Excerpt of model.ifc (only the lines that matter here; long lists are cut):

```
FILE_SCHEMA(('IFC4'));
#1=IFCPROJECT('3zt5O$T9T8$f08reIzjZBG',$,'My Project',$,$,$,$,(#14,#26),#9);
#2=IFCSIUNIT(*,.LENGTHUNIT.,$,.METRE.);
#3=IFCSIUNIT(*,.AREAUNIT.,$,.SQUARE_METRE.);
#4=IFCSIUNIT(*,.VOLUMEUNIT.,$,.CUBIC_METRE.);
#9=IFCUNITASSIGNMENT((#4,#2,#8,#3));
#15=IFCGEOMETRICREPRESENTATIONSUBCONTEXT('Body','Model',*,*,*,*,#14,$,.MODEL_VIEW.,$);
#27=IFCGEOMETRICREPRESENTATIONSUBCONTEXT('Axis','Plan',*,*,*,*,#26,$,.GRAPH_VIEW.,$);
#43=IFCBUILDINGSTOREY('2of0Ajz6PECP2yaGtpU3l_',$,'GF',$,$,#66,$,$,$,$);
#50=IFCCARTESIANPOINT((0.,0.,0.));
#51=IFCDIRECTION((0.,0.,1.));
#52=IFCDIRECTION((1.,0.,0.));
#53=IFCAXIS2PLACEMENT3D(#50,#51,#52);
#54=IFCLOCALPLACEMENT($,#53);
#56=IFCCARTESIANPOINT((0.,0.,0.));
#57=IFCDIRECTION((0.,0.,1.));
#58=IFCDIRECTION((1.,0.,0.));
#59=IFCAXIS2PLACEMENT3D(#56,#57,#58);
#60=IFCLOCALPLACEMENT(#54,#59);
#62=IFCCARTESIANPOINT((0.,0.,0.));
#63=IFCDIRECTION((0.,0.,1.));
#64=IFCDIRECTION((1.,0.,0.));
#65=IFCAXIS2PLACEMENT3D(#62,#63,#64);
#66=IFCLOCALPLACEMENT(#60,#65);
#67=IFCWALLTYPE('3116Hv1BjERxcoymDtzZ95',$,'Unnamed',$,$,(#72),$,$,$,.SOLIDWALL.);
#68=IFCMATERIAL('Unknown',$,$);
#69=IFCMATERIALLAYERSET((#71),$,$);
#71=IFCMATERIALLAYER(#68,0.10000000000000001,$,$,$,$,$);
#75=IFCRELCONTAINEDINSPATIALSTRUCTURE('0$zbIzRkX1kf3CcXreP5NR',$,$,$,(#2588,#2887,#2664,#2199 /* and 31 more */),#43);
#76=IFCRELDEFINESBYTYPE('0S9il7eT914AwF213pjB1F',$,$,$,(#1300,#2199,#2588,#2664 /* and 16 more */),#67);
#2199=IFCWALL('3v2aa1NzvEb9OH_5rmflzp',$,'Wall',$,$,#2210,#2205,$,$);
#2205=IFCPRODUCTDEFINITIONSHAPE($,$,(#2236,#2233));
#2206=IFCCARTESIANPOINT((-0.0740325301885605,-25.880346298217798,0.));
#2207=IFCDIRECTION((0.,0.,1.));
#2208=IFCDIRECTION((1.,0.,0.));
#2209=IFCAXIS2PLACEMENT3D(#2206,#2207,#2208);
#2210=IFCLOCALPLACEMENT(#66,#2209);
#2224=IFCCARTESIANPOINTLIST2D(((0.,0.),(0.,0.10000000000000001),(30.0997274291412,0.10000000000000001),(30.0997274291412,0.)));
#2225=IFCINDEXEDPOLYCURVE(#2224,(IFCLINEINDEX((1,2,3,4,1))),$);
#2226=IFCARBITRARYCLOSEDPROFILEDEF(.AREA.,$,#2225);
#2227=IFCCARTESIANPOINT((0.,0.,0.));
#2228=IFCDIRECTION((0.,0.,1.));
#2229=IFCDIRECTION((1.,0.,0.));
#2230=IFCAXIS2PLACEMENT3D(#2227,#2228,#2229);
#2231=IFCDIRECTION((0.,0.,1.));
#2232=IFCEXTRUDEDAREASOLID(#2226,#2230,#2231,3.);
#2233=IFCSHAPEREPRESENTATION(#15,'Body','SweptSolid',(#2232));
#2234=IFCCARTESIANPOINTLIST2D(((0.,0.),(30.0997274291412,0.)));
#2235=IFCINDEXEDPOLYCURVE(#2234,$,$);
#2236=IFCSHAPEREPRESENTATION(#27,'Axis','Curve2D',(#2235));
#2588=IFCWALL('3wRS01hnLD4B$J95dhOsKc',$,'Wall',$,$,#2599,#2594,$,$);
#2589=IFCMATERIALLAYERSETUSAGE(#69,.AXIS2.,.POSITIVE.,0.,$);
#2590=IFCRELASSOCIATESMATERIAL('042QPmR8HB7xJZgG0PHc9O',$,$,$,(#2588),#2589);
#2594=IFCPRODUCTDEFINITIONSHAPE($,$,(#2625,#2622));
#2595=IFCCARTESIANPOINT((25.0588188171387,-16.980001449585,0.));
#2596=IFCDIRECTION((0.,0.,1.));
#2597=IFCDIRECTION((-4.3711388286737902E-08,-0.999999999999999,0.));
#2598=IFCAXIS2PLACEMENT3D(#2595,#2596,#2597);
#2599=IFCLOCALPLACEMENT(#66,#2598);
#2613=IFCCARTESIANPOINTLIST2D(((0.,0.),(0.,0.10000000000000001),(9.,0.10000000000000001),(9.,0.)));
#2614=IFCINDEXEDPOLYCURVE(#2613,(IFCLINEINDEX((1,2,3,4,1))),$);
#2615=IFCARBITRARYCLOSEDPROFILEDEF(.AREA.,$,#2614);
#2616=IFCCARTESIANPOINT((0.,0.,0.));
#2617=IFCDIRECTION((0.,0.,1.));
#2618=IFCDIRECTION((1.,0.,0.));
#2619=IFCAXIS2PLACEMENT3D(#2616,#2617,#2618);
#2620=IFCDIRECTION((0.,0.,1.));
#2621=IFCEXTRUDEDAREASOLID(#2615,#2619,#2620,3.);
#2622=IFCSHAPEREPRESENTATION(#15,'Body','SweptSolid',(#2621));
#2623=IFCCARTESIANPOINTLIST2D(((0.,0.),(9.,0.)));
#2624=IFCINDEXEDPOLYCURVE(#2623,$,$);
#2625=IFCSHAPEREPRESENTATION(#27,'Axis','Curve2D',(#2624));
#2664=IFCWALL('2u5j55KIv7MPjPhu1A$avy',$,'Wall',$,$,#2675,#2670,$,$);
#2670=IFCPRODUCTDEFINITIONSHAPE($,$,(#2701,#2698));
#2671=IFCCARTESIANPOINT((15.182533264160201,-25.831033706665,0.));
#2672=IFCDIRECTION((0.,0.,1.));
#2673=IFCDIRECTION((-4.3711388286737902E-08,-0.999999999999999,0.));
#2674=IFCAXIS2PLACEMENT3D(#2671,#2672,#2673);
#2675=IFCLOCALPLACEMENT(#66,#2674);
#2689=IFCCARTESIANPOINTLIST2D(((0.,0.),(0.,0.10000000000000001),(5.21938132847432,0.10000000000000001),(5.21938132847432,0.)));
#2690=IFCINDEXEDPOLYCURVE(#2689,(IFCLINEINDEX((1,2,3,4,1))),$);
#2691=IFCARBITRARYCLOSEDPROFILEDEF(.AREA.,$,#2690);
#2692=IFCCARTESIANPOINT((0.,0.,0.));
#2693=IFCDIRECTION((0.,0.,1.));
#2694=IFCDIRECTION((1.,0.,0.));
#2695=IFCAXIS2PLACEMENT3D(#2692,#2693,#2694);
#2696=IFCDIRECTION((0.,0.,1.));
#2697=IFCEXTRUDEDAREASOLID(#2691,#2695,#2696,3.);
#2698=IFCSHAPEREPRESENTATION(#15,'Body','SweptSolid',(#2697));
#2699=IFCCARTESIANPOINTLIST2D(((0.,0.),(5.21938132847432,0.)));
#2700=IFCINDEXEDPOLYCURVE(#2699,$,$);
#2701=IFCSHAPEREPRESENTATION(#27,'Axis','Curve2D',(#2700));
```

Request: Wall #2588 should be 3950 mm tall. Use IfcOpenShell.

```python
import ifcopenshell
import ifcopenshell.geom
import ifcopenshell.util.representation
import ifcopenshell.util.shape
import ifcopenshell.util.unit

model = ifcopenshell.open("model.ifc")
unit_scale = ifcopenshell.util.unit.calculate_unit_scale(model)
settings = ifcopenshell.geom.settings()


def volume(element):
    """Net volume in cubic metres, openings subtracted."""
    shape = ifcopenshell.geom.create_shape(settings, element)
    return ifcopenshell.util.shape.get_volume(shape.geometry)


wall = model.by_guid("3wRS01hnLD4B$J95dhOsKc")
before = volume(wall)

body = ifcopenshell.util.representation.get_representation(wall, "Model", "Body")
solid = body.Items[0]
old_height = solid.Depth
solid.Depth = 3.95 / unit_scale
after = volume(wall)

print(f"height {old_height:g} -> {solid.Depth:g}, volume {before:.3f} -> {after:.3f} m3")

model.write("model_updated.ifc")
```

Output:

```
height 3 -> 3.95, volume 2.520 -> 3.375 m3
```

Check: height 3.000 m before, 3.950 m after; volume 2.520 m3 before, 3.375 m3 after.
